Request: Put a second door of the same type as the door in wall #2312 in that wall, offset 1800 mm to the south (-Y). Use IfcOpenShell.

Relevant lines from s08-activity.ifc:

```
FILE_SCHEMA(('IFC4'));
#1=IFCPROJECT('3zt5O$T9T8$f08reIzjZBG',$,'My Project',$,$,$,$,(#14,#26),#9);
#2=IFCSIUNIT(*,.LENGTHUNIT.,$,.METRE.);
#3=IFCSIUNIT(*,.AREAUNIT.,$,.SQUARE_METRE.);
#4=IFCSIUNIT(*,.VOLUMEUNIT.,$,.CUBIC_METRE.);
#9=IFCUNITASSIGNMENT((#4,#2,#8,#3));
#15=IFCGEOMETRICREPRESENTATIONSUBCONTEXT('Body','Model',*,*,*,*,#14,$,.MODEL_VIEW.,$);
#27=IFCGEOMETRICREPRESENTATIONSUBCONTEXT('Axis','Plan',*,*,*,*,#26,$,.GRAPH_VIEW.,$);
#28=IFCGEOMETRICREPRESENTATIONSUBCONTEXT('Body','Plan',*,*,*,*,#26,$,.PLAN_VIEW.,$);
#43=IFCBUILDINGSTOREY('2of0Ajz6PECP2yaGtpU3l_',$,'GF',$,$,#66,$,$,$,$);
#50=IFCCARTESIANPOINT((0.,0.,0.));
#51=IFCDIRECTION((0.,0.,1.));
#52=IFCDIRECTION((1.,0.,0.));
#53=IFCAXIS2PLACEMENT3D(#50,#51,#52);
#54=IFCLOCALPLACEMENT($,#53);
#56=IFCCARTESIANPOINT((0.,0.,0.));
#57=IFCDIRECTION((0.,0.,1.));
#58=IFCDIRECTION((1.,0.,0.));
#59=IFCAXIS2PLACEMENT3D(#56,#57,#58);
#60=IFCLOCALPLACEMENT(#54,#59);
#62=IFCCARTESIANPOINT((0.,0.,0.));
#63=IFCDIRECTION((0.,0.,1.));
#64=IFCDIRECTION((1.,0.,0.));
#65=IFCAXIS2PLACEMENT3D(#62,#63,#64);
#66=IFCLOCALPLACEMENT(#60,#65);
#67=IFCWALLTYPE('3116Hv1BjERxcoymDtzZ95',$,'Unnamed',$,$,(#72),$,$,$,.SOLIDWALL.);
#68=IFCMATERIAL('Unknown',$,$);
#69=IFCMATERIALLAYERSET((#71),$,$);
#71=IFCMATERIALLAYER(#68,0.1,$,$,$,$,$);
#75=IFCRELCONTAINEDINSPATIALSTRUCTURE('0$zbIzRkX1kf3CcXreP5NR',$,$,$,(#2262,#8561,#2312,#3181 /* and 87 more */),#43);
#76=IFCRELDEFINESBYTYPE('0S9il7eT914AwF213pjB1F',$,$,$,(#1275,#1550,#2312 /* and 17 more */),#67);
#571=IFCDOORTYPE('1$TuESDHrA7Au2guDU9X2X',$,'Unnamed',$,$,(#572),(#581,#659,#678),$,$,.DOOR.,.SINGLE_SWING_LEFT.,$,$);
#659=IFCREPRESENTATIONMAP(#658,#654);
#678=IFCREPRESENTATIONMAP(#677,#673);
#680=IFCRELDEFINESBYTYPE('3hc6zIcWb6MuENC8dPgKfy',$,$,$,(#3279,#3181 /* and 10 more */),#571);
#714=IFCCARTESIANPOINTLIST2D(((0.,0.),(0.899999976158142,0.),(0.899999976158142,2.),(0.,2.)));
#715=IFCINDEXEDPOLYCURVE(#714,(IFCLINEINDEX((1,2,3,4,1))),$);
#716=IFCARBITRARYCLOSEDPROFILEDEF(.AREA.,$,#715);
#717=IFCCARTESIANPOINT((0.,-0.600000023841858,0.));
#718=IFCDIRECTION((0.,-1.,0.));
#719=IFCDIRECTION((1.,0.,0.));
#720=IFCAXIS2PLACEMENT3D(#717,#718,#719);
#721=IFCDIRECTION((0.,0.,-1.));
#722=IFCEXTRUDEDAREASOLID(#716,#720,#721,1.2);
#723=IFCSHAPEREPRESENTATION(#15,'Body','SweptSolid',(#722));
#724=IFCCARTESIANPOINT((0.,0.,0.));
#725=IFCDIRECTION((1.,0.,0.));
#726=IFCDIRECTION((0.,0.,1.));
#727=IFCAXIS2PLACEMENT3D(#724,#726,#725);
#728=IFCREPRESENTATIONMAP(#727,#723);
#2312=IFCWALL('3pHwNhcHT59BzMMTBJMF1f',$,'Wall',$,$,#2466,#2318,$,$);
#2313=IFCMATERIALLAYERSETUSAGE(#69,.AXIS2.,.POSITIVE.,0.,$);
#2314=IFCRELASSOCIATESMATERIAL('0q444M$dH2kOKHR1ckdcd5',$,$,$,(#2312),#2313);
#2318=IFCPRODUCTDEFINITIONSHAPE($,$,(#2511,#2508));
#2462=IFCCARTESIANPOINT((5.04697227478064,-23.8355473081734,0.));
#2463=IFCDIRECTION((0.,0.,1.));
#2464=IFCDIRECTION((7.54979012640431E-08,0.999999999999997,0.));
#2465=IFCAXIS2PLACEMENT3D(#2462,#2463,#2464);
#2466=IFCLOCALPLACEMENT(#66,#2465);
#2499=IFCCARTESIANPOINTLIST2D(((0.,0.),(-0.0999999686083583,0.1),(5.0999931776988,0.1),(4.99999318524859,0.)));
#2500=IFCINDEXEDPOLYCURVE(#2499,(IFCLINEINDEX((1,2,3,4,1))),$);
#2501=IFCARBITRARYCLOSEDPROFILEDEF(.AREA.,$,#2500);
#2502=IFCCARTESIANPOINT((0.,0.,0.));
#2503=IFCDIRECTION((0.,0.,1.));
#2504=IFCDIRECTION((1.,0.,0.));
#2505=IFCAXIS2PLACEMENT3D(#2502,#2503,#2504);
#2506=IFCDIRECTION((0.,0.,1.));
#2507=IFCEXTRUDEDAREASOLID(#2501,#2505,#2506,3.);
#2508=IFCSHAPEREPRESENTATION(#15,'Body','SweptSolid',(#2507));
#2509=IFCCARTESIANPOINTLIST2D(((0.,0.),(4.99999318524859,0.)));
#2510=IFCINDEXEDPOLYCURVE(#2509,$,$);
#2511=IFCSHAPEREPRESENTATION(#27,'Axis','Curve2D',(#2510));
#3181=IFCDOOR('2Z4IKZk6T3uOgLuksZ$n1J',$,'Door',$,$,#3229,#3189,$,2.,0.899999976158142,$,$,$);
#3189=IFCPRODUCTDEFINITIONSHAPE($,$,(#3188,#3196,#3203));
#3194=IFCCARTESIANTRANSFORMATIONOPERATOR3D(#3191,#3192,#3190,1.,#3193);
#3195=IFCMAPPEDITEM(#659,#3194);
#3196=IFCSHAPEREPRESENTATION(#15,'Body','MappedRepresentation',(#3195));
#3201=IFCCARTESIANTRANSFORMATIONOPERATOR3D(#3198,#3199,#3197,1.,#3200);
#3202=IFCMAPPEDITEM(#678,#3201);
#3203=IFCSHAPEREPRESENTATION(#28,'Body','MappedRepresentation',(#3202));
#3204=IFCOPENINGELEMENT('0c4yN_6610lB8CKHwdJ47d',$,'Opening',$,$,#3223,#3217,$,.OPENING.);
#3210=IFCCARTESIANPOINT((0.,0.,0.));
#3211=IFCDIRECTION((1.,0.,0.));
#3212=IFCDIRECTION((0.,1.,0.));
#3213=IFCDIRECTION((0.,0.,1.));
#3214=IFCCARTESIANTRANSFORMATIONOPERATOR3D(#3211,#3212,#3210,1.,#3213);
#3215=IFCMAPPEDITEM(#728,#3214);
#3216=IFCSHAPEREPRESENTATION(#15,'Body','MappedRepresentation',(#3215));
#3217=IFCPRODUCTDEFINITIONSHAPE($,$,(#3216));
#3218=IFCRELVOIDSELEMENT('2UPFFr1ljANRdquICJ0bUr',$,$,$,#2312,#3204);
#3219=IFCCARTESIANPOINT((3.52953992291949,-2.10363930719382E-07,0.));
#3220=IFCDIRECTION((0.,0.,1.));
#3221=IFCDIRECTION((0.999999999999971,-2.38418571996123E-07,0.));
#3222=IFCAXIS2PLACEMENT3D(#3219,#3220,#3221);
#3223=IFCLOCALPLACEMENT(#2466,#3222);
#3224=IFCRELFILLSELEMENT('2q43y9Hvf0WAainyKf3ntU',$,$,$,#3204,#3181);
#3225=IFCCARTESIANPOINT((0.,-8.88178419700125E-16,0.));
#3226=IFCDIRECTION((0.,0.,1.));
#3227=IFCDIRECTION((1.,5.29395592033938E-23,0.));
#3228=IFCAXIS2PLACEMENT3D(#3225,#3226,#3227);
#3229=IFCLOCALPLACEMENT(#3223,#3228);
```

```python
import ifcopenshell
import ifcopenshell.api.feature
import ifcopenshell.api.geometry
import ifcopenshell.api.root
import ifcopenshell.geom
import ifcopenshell.util.element
import ifcopenshell.util.placement
import ifcopenshell.util.shape
import ifcopenshell.util.unit

model = ifcopenshell.open("s08-activity.ifc")
unit_scale = ifcopenshell.util.unit.calculate_unit_scale(model)
settings = ifcopenshell.geom.settings()


def volume(element):
    """Net volume in cubic metres, openings subtracted."""
    shape = ifcopenshell.geom.create_shape(settings, element)
    return ifcopenshell.util.shape.get_volume(shape.geometry)


door = model.by_id(3181)
opening = door.FillsVoids[0].RelatingOpeningElement
wall = opening.VoidsElements[0].RelatingBuildingElement
before = volume(wall)
shift = ifcopenshell.util.placement.get_local_placement(wall.ObjectPlacement)[:3, 0] * -1.8 / unit_scale

# copy_class copies the void relationship, type, container and properties, but no geometry.
new_opening = ifcopenshell.api.root.copy_class(model, product=opening)
new_opening.Representation = ifcopenshell.util.element.copy_deep(
    model, opening.Representation, exclude=["IfcGeometricRepresentationContext", "IfcRepresentationMap"]
)
new_door = ifcopenshell.api.root.copy_class(model, product=door)
new_door.Representation = ifcopenshell.util.element.copy_deep(
    model, door.Representation, exclude=["IfcGeometricRepresentationContext", "IfcRepresentationMap"]
)
ifcopenshell.api.feature.add_filling(model, opening=new_opening, element=new_door)

for old, new in ((opening, new_opening), (door, new_door)):
    matrix = ifcopenshell.util.placement.get_local_placement(old.ObjectPlacement)
    matrix[:3, 3] += shift
    ifcopenshell.api.geometry.edit_object_placement(model, product=new, matrix=matrix, is_si=False)

after = volume(wall)

print(f"wall volume {before:.3f} -> {after:.3f} m3")

model.write("s08-activity_v2.ifc")
```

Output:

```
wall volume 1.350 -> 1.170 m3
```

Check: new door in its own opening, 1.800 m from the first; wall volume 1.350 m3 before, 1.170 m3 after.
